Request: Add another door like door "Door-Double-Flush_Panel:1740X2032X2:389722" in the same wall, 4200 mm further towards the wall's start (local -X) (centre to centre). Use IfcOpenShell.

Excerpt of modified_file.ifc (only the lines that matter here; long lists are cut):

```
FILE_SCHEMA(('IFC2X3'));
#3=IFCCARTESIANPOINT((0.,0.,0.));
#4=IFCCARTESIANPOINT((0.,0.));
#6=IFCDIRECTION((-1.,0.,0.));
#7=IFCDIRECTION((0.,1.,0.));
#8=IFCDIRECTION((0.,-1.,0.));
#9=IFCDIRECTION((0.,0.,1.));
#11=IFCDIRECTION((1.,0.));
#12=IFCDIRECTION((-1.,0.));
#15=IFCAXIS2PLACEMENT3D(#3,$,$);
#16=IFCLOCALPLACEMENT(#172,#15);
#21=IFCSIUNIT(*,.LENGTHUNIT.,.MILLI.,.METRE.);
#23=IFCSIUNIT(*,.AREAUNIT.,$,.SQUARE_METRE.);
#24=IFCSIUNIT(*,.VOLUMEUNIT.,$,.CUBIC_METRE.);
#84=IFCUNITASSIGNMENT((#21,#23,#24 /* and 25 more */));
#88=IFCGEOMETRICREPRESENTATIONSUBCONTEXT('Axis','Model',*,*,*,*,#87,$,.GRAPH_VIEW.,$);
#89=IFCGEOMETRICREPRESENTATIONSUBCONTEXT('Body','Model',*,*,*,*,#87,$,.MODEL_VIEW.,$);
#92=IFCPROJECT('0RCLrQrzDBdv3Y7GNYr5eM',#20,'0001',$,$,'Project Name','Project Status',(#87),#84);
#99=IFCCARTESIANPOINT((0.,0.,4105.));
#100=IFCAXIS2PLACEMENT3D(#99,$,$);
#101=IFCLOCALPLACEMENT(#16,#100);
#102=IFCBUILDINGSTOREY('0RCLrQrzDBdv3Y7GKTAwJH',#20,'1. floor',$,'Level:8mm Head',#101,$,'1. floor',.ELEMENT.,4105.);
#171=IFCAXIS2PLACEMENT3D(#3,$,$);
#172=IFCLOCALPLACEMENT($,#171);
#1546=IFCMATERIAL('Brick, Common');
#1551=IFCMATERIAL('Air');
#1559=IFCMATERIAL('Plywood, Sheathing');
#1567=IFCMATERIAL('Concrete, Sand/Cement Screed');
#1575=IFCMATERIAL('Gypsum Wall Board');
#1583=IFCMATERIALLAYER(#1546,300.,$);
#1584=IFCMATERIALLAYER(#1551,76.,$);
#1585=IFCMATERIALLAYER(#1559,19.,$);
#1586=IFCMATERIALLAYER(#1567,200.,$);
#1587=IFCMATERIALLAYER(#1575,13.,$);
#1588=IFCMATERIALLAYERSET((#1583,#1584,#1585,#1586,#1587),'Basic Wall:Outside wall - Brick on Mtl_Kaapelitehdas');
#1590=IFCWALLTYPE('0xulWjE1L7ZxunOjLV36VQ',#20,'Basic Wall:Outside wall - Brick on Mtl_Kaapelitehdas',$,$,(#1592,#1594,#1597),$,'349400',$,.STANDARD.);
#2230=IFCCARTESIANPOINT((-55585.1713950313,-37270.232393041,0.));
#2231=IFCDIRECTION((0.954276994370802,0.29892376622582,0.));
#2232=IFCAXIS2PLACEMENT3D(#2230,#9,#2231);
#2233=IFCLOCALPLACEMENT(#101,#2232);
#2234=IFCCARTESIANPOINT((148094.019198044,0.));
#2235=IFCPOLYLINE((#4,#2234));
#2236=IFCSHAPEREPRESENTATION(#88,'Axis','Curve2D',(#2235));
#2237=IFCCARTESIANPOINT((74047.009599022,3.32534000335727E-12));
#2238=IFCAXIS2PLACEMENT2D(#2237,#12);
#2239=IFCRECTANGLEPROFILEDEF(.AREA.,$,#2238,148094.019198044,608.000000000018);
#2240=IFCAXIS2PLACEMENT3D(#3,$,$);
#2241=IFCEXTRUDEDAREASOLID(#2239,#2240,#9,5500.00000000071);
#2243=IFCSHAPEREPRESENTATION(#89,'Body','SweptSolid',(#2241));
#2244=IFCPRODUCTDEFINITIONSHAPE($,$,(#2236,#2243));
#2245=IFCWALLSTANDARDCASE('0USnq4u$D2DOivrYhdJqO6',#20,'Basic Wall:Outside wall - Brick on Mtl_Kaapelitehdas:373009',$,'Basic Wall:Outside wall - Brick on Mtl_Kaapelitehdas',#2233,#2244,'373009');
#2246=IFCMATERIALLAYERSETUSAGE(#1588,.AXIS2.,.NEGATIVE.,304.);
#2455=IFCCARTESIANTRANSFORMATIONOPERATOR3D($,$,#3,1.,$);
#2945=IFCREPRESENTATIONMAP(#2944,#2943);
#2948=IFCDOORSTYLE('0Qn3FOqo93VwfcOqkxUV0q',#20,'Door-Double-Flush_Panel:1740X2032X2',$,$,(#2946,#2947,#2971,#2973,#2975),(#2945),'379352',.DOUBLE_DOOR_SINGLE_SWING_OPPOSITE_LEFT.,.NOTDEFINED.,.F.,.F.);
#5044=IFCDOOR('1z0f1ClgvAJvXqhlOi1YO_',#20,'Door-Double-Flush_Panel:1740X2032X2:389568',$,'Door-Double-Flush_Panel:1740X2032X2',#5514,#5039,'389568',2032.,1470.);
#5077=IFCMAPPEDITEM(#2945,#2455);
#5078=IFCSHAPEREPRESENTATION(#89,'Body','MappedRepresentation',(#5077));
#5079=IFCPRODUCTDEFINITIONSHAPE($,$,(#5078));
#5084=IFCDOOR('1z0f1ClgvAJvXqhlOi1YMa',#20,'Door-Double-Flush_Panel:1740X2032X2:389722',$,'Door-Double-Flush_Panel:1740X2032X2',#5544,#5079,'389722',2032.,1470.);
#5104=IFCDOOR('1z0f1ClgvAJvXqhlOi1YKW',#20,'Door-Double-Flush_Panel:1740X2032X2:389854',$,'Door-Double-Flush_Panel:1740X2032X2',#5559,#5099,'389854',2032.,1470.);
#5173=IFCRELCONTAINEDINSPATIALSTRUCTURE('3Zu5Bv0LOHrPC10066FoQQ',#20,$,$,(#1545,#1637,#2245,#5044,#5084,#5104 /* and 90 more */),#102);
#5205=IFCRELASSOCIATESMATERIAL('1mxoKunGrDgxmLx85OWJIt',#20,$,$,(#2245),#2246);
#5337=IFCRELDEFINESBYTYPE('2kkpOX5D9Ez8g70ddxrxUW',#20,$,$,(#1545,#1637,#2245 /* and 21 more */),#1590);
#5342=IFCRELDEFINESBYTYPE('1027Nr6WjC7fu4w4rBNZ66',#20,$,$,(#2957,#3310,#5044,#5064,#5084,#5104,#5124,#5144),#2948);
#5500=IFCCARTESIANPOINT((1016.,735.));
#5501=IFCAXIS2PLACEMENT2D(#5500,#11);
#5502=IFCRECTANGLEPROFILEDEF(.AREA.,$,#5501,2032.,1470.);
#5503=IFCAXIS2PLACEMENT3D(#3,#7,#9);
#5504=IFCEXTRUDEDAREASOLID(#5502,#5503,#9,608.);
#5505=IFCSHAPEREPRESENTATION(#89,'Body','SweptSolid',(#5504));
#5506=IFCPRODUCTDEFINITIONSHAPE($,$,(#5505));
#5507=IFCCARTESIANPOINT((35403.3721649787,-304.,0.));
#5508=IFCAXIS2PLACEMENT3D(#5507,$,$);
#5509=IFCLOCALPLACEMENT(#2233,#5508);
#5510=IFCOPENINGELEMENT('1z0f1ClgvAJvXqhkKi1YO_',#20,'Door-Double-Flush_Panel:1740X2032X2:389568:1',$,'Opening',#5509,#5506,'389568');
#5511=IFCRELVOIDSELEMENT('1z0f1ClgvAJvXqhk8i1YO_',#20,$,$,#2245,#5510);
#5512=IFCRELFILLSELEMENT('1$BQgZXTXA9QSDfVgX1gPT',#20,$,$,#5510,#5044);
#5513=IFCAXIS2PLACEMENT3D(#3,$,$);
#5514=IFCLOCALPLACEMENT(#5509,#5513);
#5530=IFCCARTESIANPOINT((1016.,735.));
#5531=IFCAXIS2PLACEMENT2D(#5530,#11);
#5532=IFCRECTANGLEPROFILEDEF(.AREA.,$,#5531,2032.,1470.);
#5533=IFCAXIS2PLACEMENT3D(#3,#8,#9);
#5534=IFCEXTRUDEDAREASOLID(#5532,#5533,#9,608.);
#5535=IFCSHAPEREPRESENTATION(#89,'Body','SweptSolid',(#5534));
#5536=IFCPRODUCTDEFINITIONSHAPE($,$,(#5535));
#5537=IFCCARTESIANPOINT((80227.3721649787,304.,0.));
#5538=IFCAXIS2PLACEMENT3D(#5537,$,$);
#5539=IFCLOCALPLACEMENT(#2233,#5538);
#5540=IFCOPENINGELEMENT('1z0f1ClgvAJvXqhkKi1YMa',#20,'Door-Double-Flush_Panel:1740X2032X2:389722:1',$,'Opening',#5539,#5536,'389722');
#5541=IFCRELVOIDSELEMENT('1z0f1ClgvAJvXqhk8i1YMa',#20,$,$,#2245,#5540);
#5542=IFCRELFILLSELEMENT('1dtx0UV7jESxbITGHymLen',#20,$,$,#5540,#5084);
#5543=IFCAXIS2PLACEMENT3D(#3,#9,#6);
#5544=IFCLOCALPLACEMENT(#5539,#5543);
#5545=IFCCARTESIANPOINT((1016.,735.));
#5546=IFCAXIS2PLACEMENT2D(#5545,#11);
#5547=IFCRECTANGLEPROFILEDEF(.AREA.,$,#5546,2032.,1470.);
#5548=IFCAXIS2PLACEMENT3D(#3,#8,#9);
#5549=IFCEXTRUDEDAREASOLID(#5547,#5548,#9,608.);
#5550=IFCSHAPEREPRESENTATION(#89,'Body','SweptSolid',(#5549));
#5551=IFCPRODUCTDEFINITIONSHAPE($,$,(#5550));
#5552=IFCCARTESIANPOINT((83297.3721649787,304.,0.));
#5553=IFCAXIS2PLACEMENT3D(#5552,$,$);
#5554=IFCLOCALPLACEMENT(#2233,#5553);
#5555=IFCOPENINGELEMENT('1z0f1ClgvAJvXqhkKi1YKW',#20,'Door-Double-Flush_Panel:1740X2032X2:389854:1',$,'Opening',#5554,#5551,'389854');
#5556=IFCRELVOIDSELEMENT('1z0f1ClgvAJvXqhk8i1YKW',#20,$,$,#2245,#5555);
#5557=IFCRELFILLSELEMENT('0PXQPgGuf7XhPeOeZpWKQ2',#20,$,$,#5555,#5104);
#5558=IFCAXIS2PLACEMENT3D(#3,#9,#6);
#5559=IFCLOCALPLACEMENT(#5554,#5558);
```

```python
import ifcopenshell
import ifcopenshell.api.feature
import ifcopenshell.api.geometry
import ifcopenshell.api.root
import ifcopenshell.geom
import ifcopenshell.util.element
import ifcopenshell.util.placement
import ifcopenshell.util.shape

model = ifcopenshell.open("modified_file.ifc")
settings = ifcopenshell.geom.settings()


def volume(element):
    """Net volume in cubic metres, openings subtracted."""
    shape = ifcopenshell.geom.create_shape(settings, element)
    return ifcopenshell.util.shape.get_volume(shape.geometry)


def reuse_history(source, copy):
    """copy_class also copies each property set's owner history, people and application; keep the originals."""
    for rel in copy.IsDefinedBy:
        if rel.is_a("IfcRelDefinesByProperties") and (history := rel.RelatingPropertyDefinition.OwnerHistory):
            rel.RelatingPropertyDefinition.OwnerHistory = source.OwnerHistory
            ifcopenshell.util.element.remove_deep2(model, history)


door = model.by_guid("1z0f1ClgvAJvXqhlOi1YMa")
opening = door.FillsVoids[0].RelatingOpeningElement
wall = opening.VoidsElements[0].RelatingBuildingElement
before = volume(wall)
shift = ifcopenshell.util.placement.get_local_placement(wall.ObjectPlacement)[:3, 0] * -4200.0

# copy_class copies the void relationship, type, container and properties, but no geometry.
new_opening = ifcopenshell.api.root.copy_class(model, product=opening)
new_opening.Representation = ifcopenshell.util.element.copy_deep(
    model, opening.Representation, exclude=["IfcGeometricRepresentationContext", "IfcRepresentationMap"]
)
new_opening.Name = "Door-Double-Flush_Panel:1740X2032X2"
new_opening.Tag = None
new_door = ifcopenshell.api.root.copy_class(model, product=door)
new_door.Representation = ifcopenshell.util.element.copy_deep(
    model, door.Representation, exclude=["IfcGeometricRepresentationContext", "IfcRepresentationMap"]
)
new_door.Name = "Door-Double-Flush_Panel:1740X2032X2"
new_door.Tag = None
reuse_history(door, new_door)
fills = ifcopenshell.api.feature.add_filling(model, opening=new_opening, element=new_door)
fills.OwnerHistory = new_door.OwnerHistory  # required in IFC2X3

for old, new in ((opening, new_opening), (door, new_door)):
    matrix = ifcopenshell.util.placement.get_local_placement(old.ObjectPlacement)
    matrix[:3, 3] += shift
    ifcopenshell.api.geometry.edit_object_placement(model, product=new, matrix=matrix, is_si=False)

after = volume(wall)

print(f"wall volume {before:.3f} -> {after:.3f} m3")

model.write("modified_file_rev.ifc")
```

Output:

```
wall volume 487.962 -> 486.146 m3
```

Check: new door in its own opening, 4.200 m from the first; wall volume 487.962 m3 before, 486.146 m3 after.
